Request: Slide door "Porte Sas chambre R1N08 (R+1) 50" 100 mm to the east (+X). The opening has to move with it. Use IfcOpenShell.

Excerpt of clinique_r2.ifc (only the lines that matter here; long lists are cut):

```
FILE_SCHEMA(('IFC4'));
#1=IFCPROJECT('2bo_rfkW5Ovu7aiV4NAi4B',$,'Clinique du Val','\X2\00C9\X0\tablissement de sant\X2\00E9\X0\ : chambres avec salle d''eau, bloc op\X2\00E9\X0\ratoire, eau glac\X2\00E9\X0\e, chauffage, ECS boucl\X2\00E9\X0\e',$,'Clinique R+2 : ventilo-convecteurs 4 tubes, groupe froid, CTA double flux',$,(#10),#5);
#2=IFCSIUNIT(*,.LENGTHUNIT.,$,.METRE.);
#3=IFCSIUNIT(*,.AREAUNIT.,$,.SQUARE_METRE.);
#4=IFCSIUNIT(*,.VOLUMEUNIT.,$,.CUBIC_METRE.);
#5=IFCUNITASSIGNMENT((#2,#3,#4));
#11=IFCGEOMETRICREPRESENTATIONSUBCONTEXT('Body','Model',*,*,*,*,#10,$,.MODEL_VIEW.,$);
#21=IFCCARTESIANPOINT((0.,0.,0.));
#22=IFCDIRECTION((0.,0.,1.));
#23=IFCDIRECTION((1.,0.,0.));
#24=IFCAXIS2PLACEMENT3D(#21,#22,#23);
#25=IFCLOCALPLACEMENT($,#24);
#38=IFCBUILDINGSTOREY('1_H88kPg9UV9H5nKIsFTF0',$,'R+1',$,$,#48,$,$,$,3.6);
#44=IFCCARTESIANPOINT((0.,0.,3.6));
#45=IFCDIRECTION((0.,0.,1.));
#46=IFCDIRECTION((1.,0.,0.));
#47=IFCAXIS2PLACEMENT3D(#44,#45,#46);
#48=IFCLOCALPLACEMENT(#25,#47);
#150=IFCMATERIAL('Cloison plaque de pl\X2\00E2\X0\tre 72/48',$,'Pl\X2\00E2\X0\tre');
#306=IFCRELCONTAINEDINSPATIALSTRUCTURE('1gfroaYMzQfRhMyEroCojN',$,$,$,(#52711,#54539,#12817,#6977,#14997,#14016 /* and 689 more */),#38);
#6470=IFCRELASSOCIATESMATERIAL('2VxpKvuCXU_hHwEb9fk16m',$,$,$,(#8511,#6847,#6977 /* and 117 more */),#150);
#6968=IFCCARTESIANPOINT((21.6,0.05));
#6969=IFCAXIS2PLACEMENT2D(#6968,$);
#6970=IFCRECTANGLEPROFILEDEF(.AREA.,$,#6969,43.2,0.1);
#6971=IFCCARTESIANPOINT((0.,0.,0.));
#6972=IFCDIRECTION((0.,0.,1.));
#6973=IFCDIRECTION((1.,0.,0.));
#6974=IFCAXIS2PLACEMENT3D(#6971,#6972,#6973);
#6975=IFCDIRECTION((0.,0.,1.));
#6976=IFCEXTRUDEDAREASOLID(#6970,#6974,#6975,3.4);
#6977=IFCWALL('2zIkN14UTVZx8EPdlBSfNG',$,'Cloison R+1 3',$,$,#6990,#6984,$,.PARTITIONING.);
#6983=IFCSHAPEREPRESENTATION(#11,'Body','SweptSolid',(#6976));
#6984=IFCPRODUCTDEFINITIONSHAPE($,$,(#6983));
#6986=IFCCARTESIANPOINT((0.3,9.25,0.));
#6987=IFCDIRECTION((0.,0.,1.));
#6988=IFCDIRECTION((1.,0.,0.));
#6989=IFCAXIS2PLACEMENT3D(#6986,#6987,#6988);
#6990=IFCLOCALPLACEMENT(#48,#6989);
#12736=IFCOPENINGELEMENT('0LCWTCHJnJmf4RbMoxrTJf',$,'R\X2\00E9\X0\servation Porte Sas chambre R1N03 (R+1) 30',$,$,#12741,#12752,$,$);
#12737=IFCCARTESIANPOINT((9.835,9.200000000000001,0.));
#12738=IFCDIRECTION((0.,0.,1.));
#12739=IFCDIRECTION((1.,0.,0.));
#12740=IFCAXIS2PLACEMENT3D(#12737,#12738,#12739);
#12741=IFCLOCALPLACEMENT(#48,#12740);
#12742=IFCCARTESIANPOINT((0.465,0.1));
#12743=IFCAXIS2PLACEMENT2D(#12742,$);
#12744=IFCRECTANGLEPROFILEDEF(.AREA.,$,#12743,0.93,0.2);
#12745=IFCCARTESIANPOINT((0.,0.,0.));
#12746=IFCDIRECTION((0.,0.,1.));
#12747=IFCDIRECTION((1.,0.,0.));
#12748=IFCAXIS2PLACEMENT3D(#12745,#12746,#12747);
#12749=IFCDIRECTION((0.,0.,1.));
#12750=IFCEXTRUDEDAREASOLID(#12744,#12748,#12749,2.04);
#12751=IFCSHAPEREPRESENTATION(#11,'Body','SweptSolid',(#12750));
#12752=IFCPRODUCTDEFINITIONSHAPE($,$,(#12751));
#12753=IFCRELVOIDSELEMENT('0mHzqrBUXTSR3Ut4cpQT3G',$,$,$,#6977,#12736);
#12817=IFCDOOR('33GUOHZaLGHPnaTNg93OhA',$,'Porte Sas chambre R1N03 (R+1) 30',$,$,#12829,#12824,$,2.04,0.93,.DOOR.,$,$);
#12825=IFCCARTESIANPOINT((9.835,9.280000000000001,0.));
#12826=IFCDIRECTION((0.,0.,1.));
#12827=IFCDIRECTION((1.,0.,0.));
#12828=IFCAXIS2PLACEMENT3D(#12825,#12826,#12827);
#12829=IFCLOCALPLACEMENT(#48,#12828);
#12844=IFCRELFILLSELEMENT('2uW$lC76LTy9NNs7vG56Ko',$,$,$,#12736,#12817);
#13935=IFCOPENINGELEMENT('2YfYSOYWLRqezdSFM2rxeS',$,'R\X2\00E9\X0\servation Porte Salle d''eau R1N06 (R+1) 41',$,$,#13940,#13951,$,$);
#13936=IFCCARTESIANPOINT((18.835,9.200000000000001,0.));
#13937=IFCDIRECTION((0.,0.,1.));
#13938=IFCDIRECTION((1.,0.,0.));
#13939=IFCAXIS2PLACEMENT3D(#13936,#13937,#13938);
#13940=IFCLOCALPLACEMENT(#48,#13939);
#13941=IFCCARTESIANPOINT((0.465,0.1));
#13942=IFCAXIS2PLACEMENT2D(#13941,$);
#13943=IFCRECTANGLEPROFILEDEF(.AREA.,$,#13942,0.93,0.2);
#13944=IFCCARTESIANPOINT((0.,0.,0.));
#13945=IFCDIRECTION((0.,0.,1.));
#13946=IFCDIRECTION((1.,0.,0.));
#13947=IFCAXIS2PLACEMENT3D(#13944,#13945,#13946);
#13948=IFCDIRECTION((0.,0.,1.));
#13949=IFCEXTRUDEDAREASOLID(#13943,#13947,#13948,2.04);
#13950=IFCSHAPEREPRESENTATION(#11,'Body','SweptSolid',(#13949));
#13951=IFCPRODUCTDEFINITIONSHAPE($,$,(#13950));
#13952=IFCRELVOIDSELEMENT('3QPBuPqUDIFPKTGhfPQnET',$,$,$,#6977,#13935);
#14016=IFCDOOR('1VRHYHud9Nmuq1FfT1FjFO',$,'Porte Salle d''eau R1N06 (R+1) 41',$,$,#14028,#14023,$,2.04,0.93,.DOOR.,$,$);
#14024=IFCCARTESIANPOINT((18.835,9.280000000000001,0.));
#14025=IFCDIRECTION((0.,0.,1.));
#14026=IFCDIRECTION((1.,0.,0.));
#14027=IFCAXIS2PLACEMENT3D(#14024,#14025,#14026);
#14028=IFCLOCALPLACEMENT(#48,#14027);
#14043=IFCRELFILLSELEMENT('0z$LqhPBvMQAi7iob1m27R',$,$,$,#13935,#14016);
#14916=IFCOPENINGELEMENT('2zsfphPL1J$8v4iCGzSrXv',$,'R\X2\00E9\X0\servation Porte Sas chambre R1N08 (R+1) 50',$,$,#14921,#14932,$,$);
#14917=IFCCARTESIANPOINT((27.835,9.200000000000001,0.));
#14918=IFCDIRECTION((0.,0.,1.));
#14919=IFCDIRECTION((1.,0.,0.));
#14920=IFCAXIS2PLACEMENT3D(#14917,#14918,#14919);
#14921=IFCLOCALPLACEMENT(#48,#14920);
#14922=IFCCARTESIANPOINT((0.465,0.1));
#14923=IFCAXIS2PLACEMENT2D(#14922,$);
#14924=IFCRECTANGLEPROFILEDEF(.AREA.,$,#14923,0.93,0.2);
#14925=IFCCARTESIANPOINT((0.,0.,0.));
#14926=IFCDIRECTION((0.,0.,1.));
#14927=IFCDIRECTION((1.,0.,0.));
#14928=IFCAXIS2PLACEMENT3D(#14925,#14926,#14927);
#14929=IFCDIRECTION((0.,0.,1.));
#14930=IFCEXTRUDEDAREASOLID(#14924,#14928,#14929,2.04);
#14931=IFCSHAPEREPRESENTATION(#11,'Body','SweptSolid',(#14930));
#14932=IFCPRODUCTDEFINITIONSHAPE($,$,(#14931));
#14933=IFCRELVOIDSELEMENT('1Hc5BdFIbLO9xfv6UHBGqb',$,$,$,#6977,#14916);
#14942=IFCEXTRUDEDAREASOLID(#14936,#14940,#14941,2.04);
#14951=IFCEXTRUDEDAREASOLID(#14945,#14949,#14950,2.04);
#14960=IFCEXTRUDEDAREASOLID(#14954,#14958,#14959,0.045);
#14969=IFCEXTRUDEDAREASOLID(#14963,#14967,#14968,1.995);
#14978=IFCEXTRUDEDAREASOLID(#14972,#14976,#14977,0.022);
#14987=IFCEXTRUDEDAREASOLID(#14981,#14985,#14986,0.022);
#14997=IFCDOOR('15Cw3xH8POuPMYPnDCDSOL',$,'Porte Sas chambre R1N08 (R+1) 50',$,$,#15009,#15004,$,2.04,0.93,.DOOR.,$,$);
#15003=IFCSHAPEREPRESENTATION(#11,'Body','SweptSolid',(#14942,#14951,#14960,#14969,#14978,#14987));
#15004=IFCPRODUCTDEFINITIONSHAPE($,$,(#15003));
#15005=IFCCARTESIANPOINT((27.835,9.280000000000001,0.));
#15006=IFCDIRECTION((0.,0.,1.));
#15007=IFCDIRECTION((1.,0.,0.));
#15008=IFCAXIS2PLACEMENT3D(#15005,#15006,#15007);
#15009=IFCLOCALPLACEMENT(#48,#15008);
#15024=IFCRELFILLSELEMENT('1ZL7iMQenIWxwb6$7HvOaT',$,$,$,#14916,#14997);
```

```python
import ifcopenshell
import ifcopenshell.api.geometry
import ifcopenshell.util.placement

model = ifcopenshell.open("clinique_r2.ifc")

door = model.by_guid("15Cw3xH8POuPMYPnDCDSOL")
opening = door.FillsVoids[0].RelatingOpeningElement
wall = opening.VoidsElements[0].RelatingBuildingElement

wall_matrix = ifcopenshell.util.placement.get_local_placement(wall.ObjectPlacement)
shift = wall_matrix[:3, 0] * 0.1
before = ifcopenshell.util.placement.get_local_placement(door.ObjectPlacement)[:3, 3].copy()

# The door is not placed relative to its opening, so move both.
for product in (opening, door):
    matrix = ifcopenshell.util.placement.get_local_placement(product.ObjectPlacement)
    matrix[:3, 3] += shift
    ifcopenshell.api.geometry.edit_object_placement(model, product=product, matrix=matrix, is_si=False)

after = ifcopenshell.util.placement.get_local_placement(door.ObjectPlacement)[:3, 3]
print("door moved by", (after - before).round(3) + 0.0)

model.write("clinique_r2_v2.ifc")
```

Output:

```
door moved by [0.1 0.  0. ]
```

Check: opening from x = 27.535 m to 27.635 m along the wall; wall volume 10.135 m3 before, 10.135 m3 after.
